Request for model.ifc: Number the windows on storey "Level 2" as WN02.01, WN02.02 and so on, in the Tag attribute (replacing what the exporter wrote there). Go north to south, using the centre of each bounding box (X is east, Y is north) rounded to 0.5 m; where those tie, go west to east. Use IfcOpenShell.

First a look at what the model holds.

```python
import ifcopenshell
import ifcopenshell.util.element
import ifcopenshell.util.placement

model = ifcopenshell.open("model.ifc")
print(model.schema)
storey = next(s for s in model.by_type("IfcBuildingStorey") if s.Name == "Level 2")
windows = [e for e in ifcopenshell.util.element.get_decomposition(storey) if e.is_a("IfcWindow")]
for e in sorted(windows, key=lambda e: e.id()):
    origin = ifcopenshell.util.placement.get_local_placement(e.ObjectPlacement)[:3, 3]
    print(e.id(), e.Tag, e.Name, origin.round(2) + 0.0, sep=" | ")
```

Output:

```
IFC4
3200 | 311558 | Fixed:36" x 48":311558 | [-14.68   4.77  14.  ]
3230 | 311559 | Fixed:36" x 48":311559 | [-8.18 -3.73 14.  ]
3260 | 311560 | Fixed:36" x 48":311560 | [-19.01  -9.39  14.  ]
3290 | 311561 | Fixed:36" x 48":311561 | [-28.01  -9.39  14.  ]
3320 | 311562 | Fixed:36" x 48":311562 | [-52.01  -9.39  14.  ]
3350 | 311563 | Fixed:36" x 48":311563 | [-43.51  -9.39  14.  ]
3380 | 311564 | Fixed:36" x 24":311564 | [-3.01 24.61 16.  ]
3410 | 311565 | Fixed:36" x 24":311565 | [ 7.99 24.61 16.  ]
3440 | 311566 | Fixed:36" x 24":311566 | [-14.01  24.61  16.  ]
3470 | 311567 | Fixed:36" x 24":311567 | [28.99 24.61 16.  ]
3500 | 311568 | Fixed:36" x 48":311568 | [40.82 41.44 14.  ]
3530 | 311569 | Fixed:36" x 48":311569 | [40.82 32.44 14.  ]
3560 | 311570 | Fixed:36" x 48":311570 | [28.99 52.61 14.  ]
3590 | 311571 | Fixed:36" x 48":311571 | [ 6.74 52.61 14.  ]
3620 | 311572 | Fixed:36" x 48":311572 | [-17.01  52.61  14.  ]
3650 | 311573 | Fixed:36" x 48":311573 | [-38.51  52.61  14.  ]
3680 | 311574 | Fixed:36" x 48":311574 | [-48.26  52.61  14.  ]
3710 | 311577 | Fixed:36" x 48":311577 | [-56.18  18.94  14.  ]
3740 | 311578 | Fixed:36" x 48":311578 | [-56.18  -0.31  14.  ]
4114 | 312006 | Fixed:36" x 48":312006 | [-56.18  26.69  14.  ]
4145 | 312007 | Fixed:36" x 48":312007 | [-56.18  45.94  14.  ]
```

```python
import ifcopenshell
import ifcopenshell.geom
import ifcopenshell.util.element
import ifcopenshell.util.shape

model = ifcopenshell.open("model.ifc")
settings = ifcopenshell.geom.settings()
settings.set("use-world-coords", True)


def centre(element):
    shape = ifcopenshell.geom.create_shape(settings, element)
    return ifcopenshell.util.shape.get_bbox_centroid(shape.geometry)


storey = next(s for s in model.by_type("IfcBuildingStorey") if s.Name == "Level 2")
windows = [e for e in ifcopenshell.util.element.get_decomposition(storey) if e.is_a("IfcWindow")]

# Insertion points can sit at a corner or the storey origin, so sort by the geometry (in metres).
centres = {e: centre(e) for e in windows}
windows.sort(key=lambda e: (-round(centres[e][1] / 0.5), centres[e][0]))

for i, e in enumerate(windows, start=1):
    number = f"WN02.{i:02d}"
    e.Tag = number
    print(e.id(), number)

model.write("model_rev.ifc")
```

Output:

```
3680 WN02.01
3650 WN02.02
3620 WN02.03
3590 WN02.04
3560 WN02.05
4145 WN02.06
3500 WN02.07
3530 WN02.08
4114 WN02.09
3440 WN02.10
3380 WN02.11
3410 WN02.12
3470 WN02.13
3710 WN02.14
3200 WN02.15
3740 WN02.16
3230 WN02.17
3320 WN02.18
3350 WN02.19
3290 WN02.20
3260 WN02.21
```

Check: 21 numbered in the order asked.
